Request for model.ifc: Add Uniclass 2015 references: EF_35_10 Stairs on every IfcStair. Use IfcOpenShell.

First a look at what the model holds.

```python
import ifcopenshell

model = ifcopenshell.open("model.ifc")
print(model.schema)
print("classifications:", [c.Name for c in model.by_type("IfcClassification")])
for ifc_class in ("IfcDoor", "IfcRoof", "IfcStair", "IfcWall", "IfcWindow"):
    print(ifc_class, len(model.by_type(ifc_class)))
```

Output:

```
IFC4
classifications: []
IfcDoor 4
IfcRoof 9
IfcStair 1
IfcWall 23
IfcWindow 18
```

```python
import ifcopenshell
import ifcopenshell.api.classification

model = ifcopenshell.open("model.ifc")

system = ifcopenshell.api.classification.add_classification(model, classification="Uniclass 2015")

codes = {
    "IfcStair": ("EF_35_10", "Stairs"),
}
for ifc_class, (code, name) in codes.items():
    products = model.by_type(ifc_class)
    ifcopenshell.api.classification.add_reference(
        model, products=products, classification=system, identification=code, name=name
    )
    print(code, len(products))

model.write("model_edited.ifc")
```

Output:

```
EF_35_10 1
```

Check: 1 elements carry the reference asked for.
